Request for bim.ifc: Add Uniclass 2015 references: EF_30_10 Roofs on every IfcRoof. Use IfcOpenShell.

First a look at what the model holds.

```python
import ifcopenshell

model = ifcopenshell.open("bim.ifc")
print(model.schema)
print("classifications:", [c.Name for c in model.by_type("IfcClassification")])
for ifc_class in ("IfcDoor", "IfcRoof", "IfcStair", "IfcWall", "IfcWindow"):
    print(ifc_class, len(model.by_type(ifc_class)))
```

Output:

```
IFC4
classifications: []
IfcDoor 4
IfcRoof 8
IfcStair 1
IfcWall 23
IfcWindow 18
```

```python
import ifcopenshell
import ifcopenshell.api.classification

model = ifcopenshell.open("bim.ifc")

system = ifcopenshell.api.classification.add_classification(model, classification="Uniclass 2015")

codes = {
    "IfcRoof": ("EF_30_10", "Roofs"),
}
for ifc_class, (code, name) in codes.items():
    products = model.by_type(ifc_class)
    ifcopenshell.api.classification.add_reference(
        model, products=products, classification=system, identification=code, name=name
    )
    print(code, len(products))

model.write("bim_edited.ifc")
```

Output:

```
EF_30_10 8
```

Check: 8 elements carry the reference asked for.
